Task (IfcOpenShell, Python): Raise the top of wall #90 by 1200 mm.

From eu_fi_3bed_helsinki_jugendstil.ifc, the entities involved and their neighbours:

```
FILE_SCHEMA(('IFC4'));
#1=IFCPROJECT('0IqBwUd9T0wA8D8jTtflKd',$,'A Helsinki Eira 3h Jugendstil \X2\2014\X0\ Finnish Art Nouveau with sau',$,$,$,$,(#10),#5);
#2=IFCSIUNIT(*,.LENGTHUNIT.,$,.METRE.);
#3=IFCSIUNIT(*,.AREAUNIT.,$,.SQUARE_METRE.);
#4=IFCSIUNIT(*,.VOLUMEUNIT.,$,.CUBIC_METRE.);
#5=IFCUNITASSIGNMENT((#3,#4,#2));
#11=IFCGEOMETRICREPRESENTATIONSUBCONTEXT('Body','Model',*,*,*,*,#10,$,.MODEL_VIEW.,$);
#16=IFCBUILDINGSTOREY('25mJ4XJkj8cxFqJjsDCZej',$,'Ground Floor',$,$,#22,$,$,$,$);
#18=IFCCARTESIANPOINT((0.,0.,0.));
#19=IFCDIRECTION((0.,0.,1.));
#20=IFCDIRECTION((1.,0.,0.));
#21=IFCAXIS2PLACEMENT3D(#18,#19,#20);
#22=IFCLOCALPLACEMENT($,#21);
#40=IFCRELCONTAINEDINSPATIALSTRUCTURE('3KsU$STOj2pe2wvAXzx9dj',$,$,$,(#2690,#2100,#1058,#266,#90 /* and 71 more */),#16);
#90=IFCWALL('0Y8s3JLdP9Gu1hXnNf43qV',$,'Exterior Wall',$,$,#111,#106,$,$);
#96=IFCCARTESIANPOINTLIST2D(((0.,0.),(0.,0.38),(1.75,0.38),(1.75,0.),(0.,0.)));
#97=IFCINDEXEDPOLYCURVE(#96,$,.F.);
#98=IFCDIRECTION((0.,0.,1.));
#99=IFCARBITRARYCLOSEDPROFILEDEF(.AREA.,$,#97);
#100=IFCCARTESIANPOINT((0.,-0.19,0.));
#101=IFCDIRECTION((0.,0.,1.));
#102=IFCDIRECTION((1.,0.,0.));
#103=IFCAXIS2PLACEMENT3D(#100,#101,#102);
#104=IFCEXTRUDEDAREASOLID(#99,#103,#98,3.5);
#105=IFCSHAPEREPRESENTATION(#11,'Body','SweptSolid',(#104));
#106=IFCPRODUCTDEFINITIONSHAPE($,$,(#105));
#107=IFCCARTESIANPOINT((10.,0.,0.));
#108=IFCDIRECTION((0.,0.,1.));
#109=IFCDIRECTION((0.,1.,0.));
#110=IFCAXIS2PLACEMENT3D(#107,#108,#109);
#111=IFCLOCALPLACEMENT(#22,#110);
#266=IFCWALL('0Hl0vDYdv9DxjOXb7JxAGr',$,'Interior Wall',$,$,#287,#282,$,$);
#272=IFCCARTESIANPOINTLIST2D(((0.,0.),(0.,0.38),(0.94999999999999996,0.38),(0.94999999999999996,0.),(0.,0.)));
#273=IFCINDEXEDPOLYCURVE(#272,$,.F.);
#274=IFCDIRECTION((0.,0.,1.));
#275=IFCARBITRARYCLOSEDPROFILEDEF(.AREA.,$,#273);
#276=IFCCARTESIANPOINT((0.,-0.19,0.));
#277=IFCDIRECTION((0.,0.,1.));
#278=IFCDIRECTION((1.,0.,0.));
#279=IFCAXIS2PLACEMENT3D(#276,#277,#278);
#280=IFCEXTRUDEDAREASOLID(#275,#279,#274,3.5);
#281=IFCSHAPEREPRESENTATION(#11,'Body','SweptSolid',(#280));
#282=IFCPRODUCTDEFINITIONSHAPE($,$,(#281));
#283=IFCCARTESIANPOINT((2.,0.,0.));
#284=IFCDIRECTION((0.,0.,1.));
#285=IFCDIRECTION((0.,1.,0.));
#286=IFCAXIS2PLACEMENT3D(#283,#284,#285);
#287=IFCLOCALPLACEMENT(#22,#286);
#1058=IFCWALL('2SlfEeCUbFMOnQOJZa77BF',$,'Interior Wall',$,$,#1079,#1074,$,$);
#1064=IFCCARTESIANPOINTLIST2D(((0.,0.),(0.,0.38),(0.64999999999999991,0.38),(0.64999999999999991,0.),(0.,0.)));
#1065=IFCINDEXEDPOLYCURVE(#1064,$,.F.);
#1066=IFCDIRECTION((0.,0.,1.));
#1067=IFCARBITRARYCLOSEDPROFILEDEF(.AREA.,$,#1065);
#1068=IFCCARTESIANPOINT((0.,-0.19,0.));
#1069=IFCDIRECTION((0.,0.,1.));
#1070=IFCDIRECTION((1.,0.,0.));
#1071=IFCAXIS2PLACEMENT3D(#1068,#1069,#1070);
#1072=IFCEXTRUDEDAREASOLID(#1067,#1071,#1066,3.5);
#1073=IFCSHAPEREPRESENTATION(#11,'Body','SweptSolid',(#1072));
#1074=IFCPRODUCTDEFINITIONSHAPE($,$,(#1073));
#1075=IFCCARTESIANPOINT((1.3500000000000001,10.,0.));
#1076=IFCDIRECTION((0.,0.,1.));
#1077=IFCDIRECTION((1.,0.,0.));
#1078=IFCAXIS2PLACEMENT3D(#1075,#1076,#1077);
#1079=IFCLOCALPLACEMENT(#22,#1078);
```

```python
import ifcopenshell
import ifcopenshell.geom
import ifcopenshell.util.representation
import ifcopenshell.util.shape
import ifcopenshell.util.unit

model = ifcopenshell.open("eu_fi_3bed_helsinki_jugendstil.ifc")
unit_scale = ifcopenshell.util.unit.calculate_unit_scale(model)
settings = ifcopenshell.geom.settings()


def volume(element):
    """Net volume in cubic metres, openings subtracted."""
    shape = ifcopenshell.geom.create_shape(settings, element)
    return ifcopenshell.util.shape.get_volume(shape.geometry)


wall = model.by_id(90)
before = volume(wall)

body = ifcopenshell.util.representation.get_representation(wall, "Model", "Body")
solid = body.Items[0]
old_height = solid.Depth
solid.Depth += 1.2 / unit_scale
after = volume(wall)

print(f"height {old_height:g} -> {solid.Depth:g}, volume {before:.3f} -> {after:.3f} m3")

model.write("eu_fi_3bed_helsinki_jugendstil-out.ifc")
```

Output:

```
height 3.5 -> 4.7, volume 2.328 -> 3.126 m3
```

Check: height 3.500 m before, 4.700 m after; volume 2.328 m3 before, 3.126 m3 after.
